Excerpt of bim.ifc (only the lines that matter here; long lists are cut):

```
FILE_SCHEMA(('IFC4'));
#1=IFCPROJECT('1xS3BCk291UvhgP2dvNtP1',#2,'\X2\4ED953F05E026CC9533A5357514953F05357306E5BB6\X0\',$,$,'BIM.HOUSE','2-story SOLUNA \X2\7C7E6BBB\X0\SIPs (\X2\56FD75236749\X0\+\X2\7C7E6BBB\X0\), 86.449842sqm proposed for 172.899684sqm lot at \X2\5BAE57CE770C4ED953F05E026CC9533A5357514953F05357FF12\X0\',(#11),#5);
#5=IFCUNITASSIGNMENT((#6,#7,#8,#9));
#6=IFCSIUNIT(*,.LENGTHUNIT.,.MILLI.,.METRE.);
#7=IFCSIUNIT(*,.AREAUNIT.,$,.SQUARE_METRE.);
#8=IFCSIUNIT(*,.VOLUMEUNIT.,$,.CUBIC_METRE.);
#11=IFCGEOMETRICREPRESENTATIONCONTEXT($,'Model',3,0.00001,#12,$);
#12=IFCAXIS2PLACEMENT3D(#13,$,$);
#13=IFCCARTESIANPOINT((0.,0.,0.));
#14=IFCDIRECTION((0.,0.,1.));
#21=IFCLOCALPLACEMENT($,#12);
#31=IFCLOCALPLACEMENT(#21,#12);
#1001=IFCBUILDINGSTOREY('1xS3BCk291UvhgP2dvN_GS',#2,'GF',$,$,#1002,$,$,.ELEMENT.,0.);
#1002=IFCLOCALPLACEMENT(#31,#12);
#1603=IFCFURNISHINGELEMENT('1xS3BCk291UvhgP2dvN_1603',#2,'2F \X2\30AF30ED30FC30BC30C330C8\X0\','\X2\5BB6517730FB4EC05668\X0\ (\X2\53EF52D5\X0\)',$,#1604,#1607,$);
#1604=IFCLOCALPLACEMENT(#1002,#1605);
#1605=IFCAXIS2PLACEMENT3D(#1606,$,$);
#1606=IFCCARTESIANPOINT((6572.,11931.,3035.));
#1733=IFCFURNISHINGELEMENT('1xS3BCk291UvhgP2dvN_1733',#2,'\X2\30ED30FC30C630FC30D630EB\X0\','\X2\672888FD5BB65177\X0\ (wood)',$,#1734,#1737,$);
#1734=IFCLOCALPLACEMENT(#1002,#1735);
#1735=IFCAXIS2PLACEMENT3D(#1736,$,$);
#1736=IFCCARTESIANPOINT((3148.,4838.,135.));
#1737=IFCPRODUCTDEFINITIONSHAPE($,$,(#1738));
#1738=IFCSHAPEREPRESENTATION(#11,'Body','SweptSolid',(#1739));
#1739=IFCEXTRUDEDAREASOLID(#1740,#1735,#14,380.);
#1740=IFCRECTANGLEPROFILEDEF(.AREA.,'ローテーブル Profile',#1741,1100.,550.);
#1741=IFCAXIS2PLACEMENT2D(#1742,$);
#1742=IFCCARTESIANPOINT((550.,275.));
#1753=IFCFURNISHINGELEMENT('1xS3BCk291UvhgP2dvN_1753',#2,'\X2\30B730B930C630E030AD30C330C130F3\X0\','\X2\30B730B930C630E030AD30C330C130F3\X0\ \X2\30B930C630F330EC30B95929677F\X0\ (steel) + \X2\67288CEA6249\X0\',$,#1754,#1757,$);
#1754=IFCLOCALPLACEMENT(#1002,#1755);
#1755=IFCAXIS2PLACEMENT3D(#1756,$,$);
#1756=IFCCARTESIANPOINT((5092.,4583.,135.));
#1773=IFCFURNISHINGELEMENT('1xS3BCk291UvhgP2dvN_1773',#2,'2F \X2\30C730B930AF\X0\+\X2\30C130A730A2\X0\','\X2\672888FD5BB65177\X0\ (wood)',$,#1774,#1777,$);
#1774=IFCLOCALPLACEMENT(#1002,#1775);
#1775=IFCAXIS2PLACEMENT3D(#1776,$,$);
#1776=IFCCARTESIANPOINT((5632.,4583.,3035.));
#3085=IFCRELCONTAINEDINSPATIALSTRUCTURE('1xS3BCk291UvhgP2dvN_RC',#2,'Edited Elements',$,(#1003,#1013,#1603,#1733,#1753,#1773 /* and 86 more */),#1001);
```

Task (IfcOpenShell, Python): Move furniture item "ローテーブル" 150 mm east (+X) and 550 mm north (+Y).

```python
import ifcopenshell
import ifcopenshell.api.geometry
import ifcopenshell.util.placement

model = ifcopenshell.open("bim.ifc")

item = model.by_guid("1xS3BCk291UvhgP2dvN_1733")
matrix = ifcopenshell.util.placement.get_local_placement(item.ObjectPlacement)
matrix[0, 3] += 150.0
matrix[1, 3] += 550.0
ifcopenshell.api.geometry.edit_object_placement(model, product=item, matrix=matrix, is_si=False)

print(ifcopenshell.util.placement.get_local_placement(item.ObjectPlacement).round(3) + 0.0)

model.write("bim-out.ifc")
```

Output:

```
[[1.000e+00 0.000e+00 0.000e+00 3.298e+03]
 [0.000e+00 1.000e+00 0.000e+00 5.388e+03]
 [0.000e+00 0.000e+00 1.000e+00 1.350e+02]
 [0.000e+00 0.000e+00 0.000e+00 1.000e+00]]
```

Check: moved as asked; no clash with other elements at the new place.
